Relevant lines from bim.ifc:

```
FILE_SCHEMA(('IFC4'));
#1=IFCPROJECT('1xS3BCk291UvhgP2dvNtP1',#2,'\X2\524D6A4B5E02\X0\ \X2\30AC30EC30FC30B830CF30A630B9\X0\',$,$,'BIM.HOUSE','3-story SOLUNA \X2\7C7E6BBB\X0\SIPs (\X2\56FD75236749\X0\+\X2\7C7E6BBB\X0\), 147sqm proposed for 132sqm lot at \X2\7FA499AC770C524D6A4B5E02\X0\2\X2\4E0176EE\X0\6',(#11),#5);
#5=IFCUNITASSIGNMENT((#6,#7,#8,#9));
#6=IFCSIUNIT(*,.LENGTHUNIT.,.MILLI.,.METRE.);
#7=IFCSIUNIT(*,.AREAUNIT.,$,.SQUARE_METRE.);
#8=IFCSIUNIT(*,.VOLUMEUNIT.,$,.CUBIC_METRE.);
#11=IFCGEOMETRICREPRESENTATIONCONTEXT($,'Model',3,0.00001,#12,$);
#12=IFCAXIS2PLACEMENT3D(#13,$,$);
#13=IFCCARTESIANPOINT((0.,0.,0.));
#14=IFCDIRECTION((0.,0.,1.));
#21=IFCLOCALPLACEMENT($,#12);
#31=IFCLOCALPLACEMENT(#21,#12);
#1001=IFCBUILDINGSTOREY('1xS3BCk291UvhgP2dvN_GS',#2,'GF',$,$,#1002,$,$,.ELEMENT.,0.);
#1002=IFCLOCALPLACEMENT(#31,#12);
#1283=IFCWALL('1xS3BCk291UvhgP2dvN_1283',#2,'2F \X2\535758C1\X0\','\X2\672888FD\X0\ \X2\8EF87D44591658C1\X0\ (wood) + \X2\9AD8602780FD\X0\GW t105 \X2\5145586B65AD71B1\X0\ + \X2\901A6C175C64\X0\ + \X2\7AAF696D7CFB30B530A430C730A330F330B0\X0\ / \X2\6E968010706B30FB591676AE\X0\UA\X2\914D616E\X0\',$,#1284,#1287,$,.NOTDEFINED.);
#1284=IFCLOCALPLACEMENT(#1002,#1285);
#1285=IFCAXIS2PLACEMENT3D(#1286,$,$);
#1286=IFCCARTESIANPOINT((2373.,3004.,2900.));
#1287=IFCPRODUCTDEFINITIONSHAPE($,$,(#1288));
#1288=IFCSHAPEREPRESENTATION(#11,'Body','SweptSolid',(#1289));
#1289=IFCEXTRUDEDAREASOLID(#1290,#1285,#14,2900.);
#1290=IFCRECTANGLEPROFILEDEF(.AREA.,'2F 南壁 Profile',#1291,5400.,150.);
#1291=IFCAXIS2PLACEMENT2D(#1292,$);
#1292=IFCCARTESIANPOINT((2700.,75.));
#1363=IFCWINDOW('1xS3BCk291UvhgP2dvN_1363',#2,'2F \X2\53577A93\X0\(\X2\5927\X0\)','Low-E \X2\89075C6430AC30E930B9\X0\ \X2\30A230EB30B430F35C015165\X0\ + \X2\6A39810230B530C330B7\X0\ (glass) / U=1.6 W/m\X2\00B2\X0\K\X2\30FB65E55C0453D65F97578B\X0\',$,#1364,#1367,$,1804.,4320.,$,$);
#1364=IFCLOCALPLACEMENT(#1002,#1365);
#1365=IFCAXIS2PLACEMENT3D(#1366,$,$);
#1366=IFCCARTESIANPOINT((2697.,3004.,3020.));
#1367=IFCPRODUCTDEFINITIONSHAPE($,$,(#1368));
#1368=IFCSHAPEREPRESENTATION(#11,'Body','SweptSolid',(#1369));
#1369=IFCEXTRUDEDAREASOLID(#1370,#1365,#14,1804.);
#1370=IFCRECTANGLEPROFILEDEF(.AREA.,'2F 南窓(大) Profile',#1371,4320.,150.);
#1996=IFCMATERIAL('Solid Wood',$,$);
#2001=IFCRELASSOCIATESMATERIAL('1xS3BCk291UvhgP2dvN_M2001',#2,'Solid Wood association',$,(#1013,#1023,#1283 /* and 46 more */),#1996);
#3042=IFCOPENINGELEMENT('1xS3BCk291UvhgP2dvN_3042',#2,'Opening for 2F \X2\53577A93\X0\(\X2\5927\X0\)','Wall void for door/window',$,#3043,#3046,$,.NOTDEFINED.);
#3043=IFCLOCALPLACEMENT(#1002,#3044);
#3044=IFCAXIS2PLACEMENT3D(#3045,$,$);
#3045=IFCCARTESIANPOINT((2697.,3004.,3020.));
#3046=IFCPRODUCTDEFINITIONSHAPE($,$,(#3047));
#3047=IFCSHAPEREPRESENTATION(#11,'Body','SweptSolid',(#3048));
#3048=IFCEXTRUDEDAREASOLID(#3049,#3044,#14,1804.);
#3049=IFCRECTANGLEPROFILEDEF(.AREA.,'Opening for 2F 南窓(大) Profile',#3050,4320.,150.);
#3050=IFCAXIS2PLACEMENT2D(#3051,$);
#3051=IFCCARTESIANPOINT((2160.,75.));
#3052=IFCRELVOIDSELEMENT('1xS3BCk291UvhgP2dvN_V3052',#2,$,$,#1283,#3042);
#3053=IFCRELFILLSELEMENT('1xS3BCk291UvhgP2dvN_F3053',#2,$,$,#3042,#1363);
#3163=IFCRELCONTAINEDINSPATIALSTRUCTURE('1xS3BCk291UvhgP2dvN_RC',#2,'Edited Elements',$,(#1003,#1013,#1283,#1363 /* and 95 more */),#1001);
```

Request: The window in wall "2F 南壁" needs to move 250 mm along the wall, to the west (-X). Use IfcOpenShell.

```python
import ifcopenshell
import ifcopenshell.api.geometry
import ifcopenshell.util.placement

model = ifcopenshell.open("bim.ifc")

window = model.by_guid("1xS3BCk291UvhgP2dvN_1363")
opening = window.FillsVoids[0].RelatingOpeningElement
wall = opening.VoidsElements[0].RelatingBuildingElement

wall_matrix = ifcopenshell.util.placement.get_local_placement(wall.ObjectPlacement)
shift = wall_matrix[:3, 0] * -250.0
before = ifcopenshell.util.placement.get_local_placement(window.ObjectPlacement)[:3, 3].copy()

# The window is not placed relative to its opening, so move both.
for product in (opening, window):
    matrix = ifcopenshell.util.placement.get_local_placement(product.ObjectPlacement)
    matrix[:3, 3] += shift
    ifcopenshell.api.geometry.edit_object_placement(model, product=product, matrix=matrix, is_si=False)

after = ifcopenshell.util.placement.get_local_placement(window.ObjectPlacement)[:3, 3]
print("window moved by", (after - before).round(3) + 0.0)

model.write("bim_edited.ifc")
```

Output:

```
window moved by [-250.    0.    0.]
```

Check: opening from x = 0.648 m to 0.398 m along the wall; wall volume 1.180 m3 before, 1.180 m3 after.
